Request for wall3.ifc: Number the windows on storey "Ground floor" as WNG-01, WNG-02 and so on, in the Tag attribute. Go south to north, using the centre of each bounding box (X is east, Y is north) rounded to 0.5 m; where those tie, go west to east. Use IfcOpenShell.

First a look at what the model holds.

```python
import ifcopenshell
import ifcopenshell.util.element
import ifcopenshell.util.placement

model = ifcopenshell.open("wall3.ifc")
print(model.schema)
storey = next(s for s in model.by_type("IfcBuildingStorey") if s.Name == "Ground floor")
windows = [e for e in ifcopenshell.util.element.get_decomposition(storey) if e.is_a("IfcWindow")]
for e in sorted(windows, key=lambda e: e.id()):
    origin = ifcopenshell.util.placement.get_local_placement(e.ObjectPlacement)[:3, 3]
    print(e.id(), e.Tag, e.Name, origin.round(2) + 0.0, sep=" | ")
```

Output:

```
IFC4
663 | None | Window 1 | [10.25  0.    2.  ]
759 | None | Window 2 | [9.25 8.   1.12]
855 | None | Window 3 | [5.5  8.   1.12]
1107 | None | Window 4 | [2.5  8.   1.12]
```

```python
import ifcopenshell
import ifcopenshell.geom
import ifcopenshell.util.element
import ifcopenshell.util.shape

model = ifcopenshell.open("wall3.ifc")
settings = ifcopenshell.geom.settings()
settings.set("use-world-coords", True)


def centre(element):
    shape = ifcopenshell.geom.create_shape(settings, element)
    return ifcopenshell.util.shape.get_bbox_centroid(shape.geometry)


storey = next(s for s in model.by_type("IfcBuildingStorey") if s.Name == "Ground floor")
windows = [e for e in ifcopenshell.util.element.get_decomposition(storey) if e.is_a("IfcWindow")]

# Insertion points can sit at a corner or the storey origin, so sort by the geometry (in metres).
centres = {e: centre(e) for e in windows}
windows.sort(key=lambda e: (round(centres[e][1] / 0.5), centres[e][0]))

for i, e in enumerate(windows, start=1):
    number = f"WNG-{i:02d}"
    e.Tag = number
    print(e.id(), number)

model.write("wall3_edited.ifc")
```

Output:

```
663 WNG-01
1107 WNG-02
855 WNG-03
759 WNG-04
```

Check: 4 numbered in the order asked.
